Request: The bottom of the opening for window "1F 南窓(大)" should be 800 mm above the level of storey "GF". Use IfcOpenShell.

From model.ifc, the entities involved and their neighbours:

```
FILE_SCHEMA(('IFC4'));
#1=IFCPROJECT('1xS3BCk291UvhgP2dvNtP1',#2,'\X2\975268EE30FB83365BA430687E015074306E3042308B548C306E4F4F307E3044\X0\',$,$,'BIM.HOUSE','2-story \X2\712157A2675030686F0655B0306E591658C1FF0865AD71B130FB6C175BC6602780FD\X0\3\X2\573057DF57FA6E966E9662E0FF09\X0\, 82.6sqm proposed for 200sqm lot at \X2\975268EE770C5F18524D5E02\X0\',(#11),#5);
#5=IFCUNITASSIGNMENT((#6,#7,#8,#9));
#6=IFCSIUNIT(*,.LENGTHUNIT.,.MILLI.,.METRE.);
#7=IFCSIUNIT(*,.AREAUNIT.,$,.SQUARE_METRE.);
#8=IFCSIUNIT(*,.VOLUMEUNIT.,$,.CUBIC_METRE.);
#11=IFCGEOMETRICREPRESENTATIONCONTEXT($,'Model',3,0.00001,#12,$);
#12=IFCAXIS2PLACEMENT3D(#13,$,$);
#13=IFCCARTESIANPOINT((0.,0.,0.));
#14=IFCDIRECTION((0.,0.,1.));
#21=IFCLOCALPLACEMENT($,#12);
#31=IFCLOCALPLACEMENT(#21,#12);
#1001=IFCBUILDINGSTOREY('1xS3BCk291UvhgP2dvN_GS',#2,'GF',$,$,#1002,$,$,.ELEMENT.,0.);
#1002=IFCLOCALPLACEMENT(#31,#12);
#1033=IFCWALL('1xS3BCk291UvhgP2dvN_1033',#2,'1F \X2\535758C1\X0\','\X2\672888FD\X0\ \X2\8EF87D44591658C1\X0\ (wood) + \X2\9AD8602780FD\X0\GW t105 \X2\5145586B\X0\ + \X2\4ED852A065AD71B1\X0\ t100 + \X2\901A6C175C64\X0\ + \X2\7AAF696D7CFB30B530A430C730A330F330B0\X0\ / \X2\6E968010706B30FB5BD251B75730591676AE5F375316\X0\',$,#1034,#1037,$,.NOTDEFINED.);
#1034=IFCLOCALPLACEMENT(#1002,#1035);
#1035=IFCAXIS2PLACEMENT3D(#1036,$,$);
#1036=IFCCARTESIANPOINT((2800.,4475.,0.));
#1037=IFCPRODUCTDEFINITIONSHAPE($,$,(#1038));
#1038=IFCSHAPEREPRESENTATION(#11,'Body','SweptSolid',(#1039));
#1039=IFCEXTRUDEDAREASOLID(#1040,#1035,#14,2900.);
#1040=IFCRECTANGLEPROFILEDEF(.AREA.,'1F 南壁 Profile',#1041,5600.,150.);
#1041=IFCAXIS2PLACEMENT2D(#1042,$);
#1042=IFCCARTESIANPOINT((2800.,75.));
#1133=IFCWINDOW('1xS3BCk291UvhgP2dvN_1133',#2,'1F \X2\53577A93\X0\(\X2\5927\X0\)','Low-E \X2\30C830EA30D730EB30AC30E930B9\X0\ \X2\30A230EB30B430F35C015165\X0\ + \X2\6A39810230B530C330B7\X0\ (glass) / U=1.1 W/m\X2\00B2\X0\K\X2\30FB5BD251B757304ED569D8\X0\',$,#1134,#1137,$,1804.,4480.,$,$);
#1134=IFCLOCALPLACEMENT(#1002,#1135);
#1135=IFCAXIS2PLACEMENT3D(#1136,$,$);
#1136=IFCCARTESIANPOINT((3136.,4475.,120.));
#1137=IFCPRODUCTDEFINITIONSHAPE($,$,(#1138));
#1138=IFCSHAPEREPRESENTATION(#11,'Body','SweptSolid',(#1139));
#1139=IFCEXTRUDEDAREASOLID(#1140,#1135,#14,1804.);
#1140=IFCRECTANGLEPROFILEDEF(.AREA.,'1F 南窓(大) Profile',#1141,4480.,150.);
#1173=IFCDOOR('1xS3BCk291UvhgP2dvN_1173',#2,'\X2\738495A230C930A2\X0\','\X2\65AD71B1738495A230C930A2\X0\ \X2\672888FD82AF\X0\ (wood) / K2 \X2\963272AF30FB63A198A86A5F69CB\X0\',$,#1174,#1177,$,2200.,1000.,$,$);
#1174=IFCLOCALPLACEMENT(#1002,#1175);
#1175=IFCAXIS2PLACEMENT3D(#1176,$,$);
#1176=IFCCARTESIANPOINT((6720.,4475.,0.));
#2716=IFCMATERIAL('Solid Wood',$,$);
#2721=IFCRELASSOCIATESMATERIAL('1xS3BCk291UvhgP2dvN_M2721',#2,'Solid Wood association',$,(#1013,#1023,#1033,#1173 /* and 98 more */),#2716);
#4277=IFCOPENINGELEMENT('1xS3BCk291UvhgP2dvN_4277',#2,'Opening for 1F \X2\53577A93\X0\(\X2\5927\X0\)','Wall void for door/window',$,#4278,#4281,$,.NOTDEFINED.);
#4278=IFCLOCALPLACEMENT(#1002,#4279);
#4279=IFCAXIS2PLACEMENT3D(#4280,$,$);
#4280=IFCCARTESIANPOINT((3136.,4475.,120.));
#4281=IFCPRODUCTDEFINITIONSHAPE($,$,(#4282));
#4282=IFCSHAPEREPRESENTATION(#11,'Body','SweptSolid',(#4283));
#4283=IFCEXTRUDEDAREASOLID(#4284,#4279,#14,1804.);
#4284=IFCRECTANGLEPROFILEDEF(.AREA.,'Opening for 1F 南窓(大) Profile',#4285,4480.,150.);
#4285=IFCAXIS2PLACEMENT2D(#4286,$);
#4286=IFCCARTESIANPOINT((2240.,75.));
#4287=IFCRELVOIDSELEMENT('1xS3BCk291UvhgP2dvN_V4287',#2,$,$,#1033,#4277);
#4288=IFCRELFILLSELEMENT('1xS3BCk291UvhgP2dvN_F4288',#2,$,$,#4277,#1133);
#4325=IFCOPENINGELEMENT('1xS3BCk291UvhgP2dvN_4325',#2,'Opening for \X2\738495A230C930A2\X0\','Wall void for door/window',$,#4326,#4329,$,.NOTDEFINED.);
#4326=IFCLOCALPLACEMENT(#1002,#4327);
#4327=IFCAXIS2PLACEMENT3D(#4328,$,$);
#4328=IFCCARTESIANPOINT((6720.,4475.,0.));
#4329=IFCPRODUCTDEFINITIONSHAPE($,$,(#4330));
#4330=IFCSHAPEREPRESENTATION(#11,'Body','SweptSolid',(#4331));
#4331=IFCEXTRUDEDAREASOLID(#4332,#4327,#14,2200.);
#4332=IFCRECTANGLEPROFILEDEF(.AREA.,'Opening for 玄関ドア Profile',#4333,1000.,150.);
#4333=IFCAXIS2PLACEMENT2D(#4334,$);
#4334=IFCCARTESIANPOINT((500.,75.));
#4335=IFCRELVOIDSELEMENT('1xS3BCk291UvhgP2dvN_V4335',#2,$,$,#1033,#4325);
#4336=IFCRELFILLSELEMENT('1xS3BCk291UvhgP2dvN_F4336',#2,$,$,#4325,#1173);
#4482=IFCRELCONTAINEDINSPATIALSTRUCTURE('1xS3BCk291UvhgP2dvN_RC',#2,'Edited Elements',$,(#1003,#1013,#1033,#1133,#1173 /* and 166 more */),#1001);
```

```python
import numpy as np
import ifcopenshell
import ifcopenshell.api.geometry
import ifcopenshell.geom
import ifcopenshell.util.element
import ifcopenshell.util.placement
import ifcopenshell.util.shape
import ifcopenshell.util.unit

model = ifcopenshell.open("model.ifc")
unit_scale = ifcopenshell.util.unit.calculate_unit_scale(model)

window = model.by_guid("1xS3BCk291UvhgP2dvN_1133")
opening = window.FillsVoids[0].RelatingOpeningElement
storey = ifcopenshell.util.element.get_container(window, ifc_class="IfcBuildingStorey")
level = ifcopenshell.util.placement.get_local_placement(storey.ObjectPlacement)[2, 3]

# The opening's origin need not be at the sill, so measure its lowest point.
shape = ifcopenshell.geom.create_shape(ifcopenshell.geom.settings(), opening)
bottom = ifcopenshell.util.shape.get_shape_bottom_elevation(shape, shape.geometry) / unit_scale
dz = level + 0.8 / unit_scale - bottom

shift = np.array([0.0, 0.0, dz])
# The window is not placed relative to its opening, so move both.
for product in (opening, window):
    matrix = ifcopenshell.util.placement.get_local_placement(product.ObjectPlacement)
    matrix[:3, 3] += shift
    ifcopenshell.api.geometry.edit_object_placement(model, product=product, matrix=matrix, is_si=False)

print(f"moved by {dz * unit_scale:+.3f} m")

model.write("model_v2.ifc")
```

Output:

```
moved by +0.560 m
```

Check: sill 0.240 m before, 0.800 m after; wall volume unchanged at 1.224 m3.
